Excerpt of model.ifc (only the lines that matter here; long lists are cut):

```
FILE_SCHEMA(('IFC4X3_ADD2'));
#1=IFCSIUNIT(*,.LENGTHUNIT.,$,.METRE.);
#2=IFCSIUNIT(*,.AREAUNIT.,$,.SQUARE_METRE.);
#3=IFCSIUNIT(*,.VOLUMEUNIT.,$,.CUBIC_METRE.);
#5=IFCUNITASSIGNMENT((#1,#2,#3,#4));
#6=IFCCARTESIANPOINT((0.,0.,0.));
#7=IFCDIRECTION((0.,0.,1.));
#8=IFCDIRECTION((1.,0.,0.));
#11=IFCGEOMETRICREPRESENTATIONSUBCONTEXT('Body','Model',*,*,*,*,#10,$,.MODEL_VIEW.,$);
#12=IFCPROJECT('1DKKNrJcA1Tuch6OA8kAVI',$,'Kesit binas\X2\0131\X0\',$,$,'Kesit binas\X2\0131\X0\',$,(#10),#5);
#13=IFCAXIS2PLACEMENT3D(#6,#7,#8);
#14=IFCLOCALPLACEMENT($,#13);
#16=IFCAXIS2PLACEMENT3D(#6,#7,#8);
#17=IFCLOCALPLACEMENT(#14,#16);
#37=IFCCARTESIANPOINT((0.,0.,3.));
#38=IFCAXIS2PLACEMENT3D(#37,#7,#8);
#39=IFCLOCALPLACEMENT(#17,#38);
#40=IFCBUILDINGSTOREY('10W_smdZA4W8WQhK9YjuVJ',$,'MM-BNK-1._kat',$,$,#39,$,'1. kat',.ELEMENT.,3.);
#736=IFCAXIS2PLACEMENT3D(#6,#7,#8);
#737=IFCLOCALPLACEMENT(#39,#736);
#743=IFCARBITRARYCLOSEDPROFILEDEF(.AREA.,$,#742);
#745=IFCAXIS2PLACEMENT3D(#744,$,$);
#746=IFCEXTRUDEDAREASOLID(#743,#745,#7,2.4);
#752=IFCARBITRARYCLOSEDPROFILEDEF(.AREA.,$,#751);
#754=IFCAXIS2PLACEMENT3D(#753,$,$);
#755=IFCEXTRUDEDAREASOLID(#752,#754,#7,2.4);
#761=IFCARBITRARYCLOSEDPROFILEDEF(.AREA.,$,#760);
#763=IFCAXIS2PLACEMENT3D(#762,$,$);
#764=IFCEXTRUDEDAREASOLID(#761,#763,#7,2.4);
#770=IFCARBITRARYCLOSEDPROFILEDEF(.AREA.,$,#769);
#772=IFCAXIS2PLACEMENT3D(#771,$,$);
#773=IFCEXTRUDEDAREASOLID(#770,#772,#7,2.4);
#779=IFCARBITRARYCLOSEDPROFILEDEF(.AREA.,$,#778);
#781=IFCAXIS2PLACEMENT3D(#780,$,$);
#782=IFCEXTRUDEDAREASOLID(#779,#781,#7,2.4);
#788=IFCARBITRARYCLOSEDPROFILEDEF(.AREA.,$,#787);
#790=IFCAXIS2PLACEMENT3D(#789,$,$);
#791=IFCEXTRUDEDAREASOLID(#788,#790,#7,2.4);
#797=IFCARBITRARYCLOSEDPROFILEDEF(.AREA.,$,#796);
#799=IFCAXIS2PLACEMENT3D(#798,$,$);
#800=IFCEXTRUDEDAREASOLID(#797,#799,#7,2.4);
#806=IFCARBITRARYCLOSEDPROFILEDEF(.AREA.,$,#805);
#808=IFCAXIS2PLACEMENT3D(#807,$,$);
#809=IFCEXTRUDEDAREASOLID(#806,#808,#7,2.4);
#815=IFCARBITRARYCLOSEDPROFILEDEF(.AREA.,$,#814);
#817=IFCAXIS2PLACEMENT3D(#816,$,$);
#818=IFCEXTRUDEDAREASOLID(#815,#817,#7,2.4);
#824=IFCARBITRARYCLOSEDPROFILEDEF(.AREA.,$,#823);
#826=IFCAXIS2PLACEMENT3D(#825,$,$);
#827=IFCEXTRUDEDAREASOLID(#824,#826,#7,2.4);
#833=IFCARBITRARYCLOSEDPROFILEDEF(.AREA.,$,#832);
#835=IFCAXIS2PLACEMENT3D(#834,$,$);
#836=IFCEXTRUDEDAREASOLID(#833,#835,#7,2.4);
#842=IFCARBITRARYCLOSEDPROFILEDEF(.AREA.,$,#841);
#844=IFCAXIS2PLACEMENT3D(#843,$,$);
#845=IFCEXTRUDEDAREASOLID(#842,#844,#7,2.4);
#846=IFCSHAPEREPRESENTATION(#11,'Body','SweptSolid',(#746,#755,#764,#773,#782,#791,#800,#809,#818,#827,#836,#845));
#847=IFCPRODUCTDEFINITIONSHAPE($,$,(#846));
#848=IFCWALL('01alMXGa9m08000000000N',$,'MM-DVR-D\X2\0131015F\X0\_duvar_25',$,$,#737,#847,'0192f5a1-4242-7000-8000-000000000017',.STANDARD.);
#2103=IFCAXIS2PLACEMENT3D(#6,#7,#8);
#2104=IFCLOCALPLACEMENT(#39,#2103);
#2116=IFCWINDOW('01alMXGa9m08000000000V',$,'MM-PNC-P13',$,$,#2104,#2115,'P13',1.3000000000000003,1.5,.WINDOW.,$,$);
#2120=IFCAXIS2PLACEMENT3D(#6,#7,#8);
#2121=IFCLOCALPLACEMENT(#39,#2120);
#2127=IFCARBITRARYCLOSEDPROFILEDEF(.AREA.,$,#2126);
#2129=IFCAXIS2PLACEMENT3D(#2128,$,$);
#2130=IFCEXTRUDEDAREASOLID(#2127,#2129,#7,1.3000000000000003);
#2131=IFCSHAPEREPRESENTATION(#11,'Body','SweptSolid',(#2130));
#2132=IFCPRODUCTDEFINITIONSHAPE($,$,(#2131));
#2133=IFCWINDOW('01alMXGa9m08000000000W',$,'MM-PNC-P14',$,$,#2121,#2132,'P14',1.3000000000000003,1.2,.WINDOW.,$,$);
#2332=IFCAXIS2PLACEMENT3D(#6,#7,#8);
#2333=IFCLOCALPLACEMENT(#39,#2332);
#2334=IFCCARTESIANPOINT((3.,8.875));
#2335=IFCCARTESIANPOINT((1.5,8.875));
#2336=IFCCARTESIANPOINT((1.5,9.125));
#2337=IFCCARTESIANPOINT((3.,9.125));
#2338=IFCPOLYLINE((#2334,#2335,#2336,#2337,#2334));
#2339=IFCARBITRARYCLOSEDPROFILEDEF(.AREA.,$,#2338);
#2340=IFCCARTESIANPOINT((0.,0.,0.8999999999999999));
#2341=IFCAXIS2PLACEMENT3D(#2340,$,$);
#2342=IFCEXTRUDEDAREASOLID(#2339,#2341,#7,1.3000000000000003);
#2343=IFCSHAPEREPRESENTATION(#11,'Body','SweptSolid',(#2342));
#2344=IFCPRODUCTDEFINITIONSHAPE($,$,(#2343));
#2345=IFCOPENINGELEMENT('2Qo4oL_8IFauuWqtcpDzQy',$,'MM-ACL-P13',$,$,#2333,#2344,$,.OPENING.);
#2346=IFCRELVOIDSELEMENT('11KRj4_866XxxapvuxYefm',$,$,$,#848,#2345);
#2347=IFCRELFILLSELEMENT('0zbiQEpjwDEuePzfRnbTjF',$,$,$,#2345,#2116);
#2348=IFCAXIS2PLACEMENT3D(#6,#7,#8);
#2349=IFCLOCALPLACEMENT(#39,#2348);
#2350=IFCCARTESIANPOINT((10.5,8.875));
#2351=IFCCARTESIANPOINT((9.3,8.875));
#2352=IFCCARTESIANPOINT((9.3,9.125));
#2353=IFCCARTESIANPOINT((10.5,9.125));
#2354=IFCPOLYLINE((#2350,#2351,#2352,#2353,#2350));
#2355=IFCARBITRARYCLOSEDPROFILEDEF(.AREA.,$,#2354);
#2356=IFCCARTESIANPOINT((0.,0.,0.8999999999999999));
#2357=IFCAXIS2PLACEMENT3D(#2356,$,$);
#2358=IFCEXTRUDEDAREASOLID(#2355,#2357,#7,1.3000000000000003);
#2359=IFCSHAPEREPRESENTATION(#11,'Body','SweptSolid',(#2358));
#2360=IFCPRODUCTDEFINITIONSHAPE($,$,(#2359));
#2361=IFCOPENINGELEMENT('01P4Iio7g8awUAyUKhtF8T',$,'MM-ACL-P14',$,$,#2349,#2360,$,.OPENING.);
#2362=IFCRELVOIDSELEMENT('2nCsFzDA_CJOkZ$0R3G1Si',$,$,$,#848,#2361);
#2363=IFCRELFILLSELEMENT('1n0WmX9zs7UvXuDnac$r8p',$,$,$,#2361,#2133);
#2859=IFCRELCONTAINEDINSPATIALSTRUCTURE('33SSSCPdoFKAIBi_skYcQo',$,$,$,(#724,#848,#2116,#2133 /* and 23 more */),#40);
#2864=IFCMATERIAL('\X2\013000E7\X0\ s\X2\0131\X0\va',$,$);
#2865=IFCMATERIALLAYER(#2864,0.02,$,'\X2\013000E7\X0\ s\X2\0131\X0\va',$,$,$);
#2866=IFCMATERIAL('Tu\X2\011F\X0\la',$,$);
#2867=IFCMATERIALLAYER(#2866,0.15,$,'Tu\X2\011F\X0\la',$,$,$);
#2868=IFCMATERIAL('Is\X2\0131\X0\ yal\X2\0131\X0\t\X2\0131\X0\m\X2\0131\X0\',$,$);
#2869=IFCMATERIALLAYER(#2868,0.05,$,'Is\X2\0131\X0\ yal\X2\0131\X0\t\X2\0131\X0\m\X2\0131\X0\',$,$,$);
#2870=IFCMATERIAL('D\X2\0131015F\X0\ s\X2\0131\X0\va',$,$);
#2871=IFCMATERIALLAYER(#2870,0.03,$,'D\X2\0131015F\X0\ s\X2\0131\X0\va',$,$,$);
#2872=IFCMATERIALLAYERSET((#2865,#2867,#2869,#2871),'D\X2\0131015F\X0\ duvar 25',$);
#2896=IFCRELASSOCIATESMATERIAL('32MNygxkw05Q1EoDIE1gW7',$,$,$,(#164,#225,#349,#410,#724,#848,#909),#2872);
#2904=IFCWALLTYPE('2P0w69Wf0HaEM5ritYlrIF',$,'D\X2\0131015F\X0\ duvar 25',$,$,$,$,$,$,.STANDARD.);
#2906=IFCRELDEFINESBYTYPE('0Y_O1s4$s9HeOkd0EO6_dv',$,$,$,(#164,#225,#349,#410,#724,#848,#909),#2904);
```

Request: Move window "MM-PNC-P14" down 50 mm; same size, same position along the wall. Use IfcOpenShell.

```python
import numpy as np
import ifcopenshell
import ifcopenshell.api.geometry
import ifcopenshell.util.placement
import ifcopenshell.util.unit

model = ifcopenshell.open("model.ifc")
unit_scale = ifcopenshell.util.unit.calculate_unit_scale(model)

window = model.by_guid("01alMXGa9m08000000000W")
opening = window.FillsVoids[0].RelatingOpeningElement
dz = -0.05 / unit_scale

shift = np.array([0.0, 0.0, dz])
# The window is not placed relative to its opening, so move both.
for product in (opening, window):
    matrix = ifcopenshell.util.placement.get_local_placement(product.ObjectPlacement)
    matrix[:3, 3] += shift
    ifcopenshell.api.geometry.edit_object_placement(model, product=product, matrix=matrix, is_si=False)

print(f"moved by {dz * unit_scale:+.3f} m")

model.write("model_v2.ifc")
```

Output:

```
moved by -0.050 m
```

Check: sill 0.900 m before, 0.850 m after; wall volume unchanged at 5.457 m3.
